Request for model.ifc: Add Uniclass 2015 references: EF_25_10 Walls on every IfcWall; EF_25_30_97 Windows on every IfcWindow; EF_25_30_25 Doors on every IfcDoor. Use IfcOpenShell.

First a look at what the model holds.

```python
import ifcopenshell

model = ifcopenshell.open("model.ifc")
print(model.schema)
print("classifications:", [c.Name for c in model.by_type("IfcClassification")])
for ifc_class in ("IfcDoor", "IfcRoof", "IfcStair", "IfcWall", "IfcWindow"):
    print(ifc_class, len(model.by_type(ifc_class)))
```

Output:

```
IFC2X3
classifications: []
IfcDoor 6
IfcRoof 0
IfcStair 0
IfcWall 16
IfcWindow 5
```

```python
import ifcopenshell
import ifcopenshell.api.classification

model = ifcopenshell.open("model.ifc")

# IFC2X3 requires Source and Edition and has no link from the project to the system.
system = model.create_entity("IfcClassification", Source="NBS", Edition="2015", Name="Uniclass 2015")

codes = {
    "IfcWall": ("EF_25_10", "Walls"),
    "IfcWindow": ("EF_25_30_97", "Windows"),
    "IfcDoor": ("EF_25_30_25", "Doors"),
}
for ifc_class, (code, name) in codes.items():
    products = model.by_type(ifc_class)
    ifcopenshell.api.classification.add_reference(
        model, products=products, classification=system, identification=code, name=name
    )
    print(code, len(products))

model.write("model_updated.ifc")
```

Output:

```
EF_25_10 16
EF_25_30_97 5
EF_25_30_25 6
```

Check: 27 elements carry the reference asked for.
